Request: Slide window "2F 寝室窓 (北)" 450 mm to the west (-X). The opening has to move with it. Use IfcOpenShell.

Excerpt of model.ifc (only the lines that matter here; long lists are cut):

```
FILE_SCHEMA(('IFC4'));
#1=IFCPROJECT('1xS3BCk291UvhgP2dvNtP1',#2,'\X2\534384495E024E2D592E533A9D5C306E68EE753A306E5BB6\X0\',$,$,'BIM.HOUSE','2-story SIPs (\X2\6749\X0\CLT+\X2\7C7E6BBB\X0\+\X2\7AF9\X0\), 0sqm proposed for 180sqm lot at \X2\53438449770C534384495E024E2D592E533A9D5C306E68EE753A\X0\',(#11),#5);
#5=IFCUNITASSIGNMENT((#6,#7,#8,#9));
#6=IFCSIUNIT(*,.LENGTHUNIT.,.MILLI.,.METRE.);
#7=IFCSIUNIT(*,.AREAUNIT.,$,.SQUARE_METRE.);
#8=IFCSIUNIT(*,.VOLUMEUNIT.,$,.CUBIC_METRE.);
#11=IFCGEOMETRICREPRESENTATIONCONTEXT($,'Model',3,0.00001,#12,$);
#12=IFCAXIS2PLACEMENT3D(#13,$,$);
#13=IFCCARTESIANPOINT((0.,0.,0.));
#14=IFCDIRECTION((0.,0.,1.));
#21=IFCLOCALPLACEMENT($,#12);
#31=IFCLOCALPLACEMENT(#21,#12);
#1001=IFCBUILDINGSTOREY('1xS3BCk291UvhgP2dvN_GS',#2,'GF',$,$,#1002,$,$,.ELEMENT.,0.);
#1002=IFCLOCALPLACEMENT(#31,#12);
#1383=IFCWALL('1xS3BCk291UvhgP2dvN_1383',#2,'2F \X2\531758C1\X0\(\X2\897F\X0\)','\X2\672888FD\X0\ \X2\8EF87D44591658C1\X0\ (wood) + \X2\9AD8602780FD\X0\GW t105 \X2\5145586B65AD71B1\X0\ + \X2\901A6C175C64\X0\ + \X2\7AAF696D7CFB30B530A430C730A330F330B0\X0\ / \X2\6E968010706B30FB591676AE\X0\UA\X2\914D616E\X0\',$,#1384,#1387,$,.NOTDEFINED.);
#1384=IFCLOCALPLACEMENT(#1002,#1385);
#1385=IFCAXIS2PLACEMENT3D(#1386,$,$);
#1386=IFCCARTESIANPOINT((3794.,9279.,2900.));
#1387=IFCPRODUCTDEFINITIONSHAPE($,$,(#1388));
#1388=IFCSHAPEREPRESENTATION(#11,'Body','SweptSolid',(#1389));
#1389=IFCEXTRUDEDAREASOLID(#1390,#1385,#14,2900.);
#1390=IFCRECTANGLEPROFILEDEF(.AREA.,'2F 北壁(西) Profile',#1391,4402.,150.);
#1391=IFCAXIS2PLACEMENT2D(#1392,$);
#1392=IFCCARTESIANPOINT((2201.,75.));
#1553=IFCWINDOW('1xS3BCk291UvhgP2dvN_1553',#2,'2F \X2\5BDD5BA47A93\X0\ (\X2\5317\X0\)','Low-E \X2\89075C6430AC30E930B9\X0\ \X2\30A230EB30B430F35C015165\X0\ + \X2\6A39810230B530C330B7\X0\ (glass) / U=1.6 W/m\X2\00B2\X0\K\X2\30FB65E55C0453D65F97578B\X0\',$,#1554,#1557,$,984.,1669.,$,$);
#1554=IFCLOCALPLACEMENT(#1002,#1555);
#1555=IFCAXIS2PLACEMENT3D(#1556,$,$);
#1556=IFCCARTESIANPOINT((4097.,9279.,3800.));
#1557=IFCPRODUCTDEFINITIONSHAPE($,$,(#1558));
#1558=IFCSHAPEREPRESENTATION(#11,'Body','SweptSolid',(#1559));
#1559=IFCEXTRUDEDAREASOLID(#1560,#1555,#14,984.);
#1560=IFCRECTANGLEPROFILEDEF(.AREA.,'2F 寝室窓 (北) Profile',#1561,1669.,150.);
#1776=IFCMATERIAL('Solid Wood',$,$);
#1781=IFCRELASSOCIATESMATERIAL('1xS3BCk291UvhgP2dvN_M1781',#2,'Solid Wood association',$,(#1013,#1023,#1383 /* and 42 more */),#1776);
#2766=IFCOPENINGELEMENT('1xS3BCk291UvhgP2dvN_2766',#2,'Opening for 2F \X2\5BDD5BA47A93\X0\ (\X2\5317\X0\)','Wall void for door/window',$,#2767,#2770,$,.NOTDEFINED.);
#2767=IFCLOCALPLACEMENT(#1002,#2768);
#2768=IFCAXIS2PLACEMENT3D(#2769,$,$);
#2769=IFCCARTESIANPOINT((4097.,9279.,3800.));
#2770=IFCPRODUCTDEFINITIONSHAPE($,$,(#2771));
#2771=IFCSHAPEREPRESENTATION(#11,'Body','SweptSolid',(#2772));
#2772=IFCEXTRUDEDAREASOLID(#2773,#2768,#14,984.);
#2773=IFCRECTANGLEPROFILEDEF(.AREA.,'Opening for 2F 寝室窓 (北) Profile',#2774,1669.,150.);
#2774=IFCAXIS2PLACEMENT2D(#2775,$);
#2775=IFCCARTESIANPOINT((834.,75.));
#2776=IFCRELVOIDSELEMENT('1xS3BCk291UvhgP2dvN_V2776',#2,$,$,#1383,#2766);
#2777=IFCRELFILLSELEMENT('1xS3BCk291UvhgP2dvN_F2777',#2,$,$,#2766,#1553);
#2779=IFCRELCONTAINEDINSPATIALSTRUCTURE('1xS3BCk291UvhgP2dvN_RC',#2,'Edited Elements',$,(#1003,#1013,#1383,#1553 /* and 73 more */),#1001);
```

```python
import ifcopenshell
import ifcopenshell.api.geometry
import ifcopenshell.util.placement
import ifcopenshell.util.unit

model = ifcopenshell.open("model.ifc")
unit_scale = ifcopenshell.util.unit.calculate_unit_scale(model)

window = model.by_id(1553)
opening = window.FillsVoids[0].RelatingOpeningElement
wall = opening.VoidsElements[0].RelatingBuildingElement

wall_matrix = ifcopenshell.util.placement.get_local_placement(wall.ObjectPlacement)
shift = wall_matrix[:3, 0] * -0.45 / unit_scale
before = ifcopenshell.util.placement.get_local_placement(window.ObjectPlacement)[:3, 3].copy()

# The window is not placed relative to its opening, so move both.
for product in (opening, window):
    matrix = ifcopenshell.util.placement.get_local_placement(product.ObjectPlacement)
    matrix[:3, 3] += shift
    ifcopenshell.api.geometry.edit_object_placement(model, product=product, matrix=matrix, is_si=False)

after = ifcopenshell.util.placement.get_local_placement(window.ObjectPlacement)[:3, 3]
print("window moved by", (after - before).round(3) + 0.0)

model.write("model_updated.ifc")
```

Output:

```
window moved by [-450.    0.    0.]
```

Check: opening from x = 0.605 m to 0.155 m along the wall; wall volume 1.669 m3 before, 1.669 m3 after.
